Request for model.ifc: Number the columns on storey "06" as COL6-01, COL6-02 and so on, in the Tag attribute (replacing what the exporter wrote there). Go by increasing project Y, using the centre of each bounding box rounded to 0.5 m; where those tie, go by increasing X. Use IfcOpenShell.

First a look at what the model holds.

```python
import ifcopenshell
import ifcopenshell.util.element
import ifcopenshell.util.placement

model = ifcopenshell.open("model.ifc")
print(model.schema)
storey = next(s for s in model.by_type("IfcBuildingStorey") if s.Name == "06")
columns = [e for e in ifcopenshell.util.element.get_decomposition(storey) if e.is_a("IfcColumn")]
for e in sorted(columns, key=lambda e: e.id()):
    origin = ifcopenshell.util.placement.get_local_placement(e.ObjectPlacement)[:3, 3]
    print(e.id(), e.Tag, e.Name, origin.round(2) + 0.0, sep=" | ")
```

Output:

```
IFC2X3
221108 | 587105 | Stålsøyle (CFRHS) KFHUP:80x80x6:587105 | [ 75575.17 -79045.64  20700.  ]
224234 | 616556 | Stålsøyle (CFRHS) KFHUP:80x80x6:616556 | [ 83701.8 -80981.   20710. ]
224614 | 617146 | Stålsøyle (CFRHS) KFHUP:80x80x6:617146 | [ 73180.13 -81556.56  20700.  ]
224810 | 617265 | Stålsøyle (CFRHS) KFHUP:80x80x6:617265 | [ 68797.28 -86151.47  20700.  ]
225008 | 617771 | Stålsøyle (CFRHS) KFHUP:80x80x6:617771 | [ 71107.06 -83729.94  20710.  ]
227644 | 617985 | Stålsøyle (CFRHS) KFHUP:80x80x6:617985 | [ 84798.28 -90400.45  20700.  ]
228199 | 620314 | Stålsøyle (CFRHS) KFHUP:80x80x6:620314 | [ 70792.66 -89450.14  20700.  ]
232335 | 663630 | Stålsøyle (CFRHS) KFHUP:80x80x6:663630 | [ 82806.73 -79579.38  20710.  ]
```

```python
import ifcopenshell
import ifcopenshell.geom
import ifcopenshell.util.element
import ifcopenshell.util.shape

model = ifcopenshell.open("model.ifc")
settings = ifcopenshell.geom.settings()
settings.set("use-world-coords", True)


def centre(element):
    shape = ifcopenshell.geom.create_shape(settings, element)
    return ifcopenshell.util.shape.get_bbox_centroid(shape.geometry)


storey = next(s for s in model.by_type("IfcBuildingStorey") if s.Name == "06")
columns = [e for e in ifcopenshell.util.element.get_decomposition(storey) if e.is_a("IfcColumn")]

# Insertion points can sit at a corner or the storey origin, so sort by the geometry (in metres).
centres = {e: centre(e) for e in columns}
columns.sort(key=lambda e: (round(centres[e][1] / 0.5), centres[e][0]))

for i, e in enumerate(columns, start=1):
    number = f"COL6-{i:02d}"
    e.Tag = number
    print(e.id(), number)

model.write("model_v2.ifc")
```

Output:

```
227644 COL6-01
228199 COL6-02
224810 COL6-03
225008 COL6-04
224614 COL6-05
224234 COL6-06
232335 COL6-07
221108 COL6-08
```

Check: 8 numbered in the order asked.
